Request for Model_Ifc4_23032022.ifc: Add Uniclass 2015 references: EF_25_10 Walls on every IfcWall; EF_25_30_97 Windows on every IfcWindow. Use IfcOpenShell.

First a look at what the model holds.

```python
import ifcopenshell

model = ifcopenshell.open("Model_Ifc4_23032022.ifc")
print(model.schema)
print("classifications:", [c.Name for c in model.by_type("IfcClassification")])
for ifc_class in ("IfcDoor", "IfcRoof", "IfcStair", "IfcWall", "IfcWindow"):
    print(ifc_class, len(model.by_type(ifc_class)))
```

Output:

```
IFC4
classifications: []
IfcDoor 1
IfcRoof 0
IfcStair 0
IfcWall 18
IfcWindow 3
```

```python
import ifcopenshell
import ifcopenshell.api.classification

model = ifcopenshell.open("Model_Ifc4_23032022.ifc")

system = ifcopenshell.api.classification.add_classification(model, classification="Uniclass 2015")

codes = {
    "IfcWall": ("EF_25_10", "Walls"),
    "IfcWindow": ("EF_25_30_97", "Windows"),
}
for ifc_class, (code, name) in codes.items():
    products = model.by_type(ifc_class)
    ifcopenshell.api.classification.add_reference(
        model, products=products, classification=system, identification=code, name=name
    )
    print(code, len(products))

model.write("Model_Ifc4_23032022-out.ifc")
```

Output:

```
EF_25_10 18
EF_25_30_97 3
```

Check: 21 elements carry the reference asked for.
